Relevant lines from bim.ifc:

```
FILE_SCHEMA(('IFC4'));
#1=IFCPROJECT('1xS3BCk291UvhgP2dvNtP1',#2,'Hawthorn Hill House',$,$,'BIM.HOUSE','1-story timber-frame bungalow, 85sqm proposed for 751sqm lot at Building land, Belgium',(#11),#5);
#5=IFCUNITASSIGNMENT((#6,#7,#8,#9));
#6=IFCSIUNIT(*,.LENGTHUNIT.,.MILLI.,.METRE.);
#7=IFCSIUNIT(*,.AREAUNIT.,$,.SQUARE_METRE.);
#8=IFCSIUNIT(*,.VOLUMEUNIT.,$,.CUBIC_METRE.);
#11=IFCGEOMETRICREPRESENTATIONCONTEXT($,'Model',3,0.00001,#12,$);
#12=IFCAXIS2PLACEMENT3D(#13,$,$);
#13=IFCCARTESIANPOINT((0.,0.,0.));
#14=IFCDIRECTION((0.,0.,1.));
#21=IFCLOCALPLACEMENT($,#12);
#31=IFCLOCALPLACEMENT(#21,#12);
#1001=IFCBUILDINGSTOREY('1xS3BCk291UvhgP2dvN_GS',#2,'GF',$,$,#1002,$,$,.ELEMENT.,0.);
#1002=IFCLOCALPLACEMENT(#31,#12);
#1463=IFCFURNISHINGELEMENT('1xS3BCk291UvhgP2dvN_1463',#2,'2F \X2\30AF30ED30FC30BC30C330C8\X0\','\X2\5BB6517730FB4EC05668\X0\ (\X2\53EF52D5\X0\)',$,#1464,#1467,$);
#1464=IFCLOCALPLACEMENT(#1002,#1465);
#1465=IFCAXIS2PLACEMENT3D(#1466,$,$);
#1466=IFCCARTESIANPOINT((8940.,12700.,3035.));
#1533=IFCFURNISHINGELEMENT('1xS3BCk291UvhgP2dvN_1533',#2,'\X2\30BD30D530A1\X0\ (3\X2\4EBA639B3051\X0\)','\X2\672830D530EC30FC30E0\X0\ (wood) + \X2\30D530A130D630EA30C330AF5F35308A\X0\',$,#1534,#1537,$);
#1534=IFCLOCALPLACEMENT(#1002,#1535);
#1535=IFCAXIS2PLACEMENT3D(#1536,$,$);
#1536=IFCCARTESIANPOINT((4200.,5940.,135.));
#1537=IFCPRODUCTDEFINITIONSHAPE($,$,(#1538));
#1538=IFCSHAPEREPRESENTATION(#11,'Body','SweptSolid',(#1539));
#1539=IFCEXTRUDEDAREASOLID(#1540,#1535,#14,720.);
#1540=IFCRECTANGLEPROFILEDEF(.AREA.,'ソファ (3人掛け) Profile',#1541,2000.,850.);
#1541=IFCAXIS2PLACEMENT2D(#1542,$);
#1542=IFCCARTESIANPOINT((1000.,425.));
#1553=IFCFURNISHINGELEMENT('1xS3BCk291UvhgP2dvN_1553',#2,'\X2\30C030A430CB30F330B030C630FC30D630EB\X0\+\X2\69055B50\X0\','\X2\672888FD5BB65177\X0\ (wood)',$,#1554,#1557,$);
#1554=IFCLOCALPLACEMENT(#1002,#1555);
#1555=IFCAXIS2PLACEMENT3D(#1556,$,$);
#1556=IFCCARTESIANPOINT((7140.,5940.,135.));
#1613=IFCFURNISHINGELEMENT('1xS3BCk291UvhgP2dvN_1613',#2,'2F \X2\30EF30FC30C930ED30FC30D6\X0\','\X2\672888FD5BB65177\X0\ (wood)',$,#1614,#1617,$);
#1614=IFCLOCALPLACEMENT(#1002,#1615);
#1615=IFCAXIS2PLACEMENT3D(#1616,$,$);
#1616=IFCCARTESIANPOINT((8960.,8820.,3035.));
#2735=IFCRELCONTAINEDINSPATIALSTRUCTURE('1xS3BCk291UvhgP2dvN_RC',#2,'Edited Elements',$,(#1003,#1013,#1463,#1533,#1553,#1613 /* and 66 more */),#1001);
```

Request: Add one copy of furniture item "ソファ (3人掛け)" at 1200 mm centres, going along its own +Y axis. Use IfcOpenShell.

```python
import ifcopenshell
import ifcopenshell.api.geometry
import ifcopenshell.api.root
import ifcopenshell.util.element
import ifcopenshell.util.placement
import ifcopenshell.util.unit

model = ifcopenshell.open("bim.ifc")
unit_scale = ifcopenshell.util.unit.calculate_unit_scale(model)


def reuse_history(source, copy):
    """copy_class also copies each property set's owner history, people and application; keep the originals."""
    for rel in copy.IsDefinedBy:
        if rel.is_a("IfcRelDefinesByProperties") and (history := rel.RelatingPropertyDefinition.OwnerHistory):
            rel.RelatingPropertyDefinition.OwnerHistory = source.OwnerHistory
            ifcopenshell.util.element.remove_deep2(model, history)


source = model.by_guid("1xS3BCk291UvhgP2dvN_1533")
base = ifcopenshell.util.placement.get_local_placement(source.ObjectPlacement)
step = base[:3, 1] * 1.2 / unit_scale

for i in range(1, 2):
    copy = ifcopenshell.api.root.copy_class(model, product=source)
    copy.Representation = ifcopenshell.util.element.copy_deep(
        model, source.Representation, exclude=["IfcGeometricRepresentationContext", "IfcRepresentationMap"]
    )
    reuse_history(source, copy)
    matrix = base.copy()
    matrix[:3, 3] += i * step
    print("added at", matrix[:3, 3].round(3) + 0.0)
    ifcopenshell.api.geometry.edit_object_placement(model, product=copy, matrix=matrix, is_si=False)

model.write("bim_edited.ifc")
```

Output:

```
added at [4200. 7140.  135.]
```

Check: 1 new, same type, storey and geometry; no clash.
